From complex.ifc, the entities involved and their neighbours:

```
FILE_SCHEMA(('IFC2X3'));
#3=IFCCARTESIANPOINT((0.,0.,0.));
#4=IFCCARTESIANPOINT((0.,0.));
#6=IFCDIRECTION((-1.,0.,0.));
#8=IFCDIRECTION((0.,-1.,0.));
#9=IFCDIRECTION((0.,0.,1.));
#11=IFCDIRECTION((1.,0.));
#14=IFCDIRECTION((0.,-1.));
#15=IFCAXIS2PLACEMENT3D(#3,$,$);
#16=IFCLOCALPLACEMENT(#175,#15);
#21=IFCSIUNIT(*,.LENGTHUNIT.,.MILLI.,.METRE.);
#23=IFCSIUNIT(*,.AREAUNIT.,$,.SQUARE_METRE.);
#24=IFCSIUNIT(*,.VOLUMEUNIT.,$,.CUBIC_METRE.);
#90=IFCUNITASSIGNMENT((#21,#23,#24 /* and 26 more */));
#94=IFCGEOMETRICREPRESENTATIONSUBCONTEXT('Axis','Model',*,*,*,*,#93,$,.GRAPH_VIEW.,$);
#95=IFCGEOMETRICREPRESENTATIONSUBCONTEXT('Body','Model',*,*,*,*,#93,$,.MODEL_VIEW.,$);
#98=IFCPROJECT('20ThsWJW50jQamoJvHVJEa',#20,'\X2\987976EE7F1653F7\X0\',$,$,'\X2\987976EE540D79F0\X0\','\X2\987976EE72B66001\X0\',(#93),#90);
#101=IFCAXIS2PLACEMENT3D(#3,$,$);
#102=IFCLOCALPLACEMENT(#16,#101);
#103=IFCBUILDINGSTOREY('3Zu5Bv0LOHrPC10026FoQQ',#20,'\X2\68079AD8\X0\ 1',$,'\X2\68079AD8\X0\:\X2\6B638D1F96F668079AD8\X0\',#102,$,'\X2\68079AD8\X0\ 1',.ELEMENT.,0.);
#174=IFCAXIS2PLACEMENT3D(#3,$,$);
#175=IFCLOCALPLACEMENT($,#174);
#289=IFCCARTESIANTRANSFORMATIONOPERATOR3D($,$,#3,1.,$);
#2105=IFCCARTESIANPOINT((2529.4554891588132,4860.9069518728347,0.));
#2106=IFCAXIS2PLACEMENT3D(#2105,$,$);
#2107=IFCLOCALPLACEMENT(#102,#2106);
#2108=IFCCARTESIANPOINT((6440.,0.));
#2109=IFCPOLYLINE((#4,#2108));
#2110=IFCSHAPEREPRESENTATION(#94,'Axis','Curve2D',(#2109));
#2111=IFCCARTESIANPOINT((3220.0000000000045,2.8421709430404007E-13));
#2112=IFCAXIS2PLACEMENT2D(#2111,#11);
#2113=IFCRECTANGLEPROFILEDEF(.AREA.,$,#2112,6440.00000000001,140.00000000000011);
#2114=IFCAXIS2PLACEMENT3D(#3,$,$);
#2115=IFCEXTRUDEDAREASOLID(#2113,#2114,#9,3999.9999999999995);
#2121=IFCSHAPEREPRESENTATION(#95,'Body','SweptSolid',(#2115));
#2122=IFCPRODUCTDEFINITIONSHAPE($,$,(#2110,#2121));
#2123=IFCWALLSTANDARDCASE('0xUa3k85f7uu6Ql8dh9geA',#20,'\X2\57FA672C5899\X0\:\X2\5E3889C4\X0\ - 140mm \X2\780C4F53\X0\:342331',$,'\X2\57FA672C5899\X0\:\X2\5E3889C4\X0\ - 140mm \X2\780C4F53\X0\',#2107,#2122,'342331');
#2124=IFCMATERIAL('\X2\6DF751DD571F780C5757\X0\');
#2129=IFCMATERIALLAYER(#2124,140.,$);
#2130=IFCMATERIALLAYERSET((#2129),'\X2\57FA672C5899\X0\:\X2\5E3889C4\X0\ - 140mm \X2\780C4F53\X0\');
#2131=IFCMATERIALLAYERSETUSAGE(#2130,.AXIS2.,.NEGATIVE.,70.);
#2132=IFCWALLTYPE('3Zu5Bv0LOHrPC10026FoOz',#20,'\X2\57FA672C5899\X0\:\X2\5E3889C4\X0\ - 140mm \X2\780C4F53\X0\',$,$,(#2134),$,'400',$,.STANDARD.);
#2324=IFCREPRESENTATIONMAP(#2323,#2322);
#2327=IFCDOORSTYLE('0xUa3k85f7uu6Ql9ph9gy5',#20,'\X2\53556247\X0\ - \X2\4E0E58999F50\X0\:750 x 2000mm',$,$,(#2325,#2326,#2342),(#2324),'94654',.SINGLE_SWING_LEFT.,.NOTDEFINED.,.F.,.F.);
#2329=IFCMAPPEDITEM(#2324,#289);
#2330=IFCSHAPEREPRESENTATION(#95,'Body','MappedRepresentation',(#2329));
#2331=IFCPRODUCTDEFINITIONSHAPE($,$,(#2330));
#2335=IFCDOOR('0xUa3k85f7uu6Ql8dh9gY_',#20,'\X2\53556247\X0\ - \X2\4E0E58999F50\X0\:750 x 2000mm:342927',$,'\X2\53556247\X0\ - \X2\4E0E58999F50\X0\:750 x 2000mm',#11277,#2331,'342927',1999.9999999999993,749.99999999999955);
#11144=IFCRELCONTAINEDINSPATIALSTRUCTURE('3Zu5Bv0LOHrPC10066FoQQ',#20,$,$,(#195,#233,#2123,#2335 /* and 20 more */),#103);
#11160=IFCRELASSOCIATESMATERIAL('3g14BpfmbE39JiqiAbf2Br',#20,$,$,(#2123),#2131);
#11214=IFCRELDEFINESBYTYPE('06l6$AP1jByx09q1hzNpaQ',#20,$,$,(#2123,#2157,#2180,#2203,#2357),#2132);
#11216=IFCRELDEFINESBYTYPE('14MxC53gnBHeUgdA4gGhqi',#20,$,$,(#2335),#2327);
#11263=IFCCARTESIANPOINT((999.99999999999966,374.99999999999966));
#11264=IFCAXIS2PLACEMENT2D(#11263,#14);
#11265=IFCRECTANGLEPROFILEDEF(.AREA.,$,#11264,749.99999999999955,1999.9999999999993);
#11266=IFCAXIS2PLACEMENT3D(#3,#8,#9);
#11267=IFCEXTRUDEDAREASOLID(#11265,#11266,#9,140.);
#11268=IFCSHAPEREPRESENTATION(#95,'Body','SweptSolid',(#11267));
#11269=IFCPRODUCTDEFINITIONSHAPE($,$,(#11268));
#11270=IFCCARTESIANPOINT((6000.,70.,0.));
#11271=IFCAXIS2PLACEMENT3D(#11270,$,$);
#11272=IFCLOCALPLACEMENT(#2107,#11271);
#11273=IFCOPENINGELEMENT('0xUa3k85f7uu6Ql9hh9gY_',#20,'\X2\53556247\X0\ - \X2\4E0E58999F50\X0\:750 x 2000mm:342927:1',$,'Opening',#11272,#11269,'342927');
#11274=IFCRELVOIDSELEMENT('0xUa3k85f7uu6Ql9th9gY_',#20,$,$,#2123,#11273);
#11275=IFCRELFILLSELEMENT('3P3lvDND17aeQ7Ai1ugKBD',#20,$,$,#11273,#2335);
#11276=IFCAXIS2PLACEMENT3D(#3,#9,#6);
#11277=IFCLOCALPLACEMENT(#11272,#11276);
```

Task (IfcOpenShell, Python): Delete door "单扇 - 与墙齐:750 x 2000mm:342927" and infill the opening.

```python
import ifcopenshell
import ifcopenshell.api.feature
import ifcopenshell.api.root
import ifcopenshell.geom
import ifcopenshell.util.shape

model = ifcopenshell.open("complex.ifc")
settings = ifcopenshell.geom.settings()


def volume(element):
    """Net volume in cubic metres, openings subtracted."""
    shape = ifcopenshell.geom.create_shape(settings, element)
    return ifcopenshell.util.shape.get_volume(shape.geometry)


door = model.by_id(2335)
opening = door.FillsVoids[0].RelatingOpeningElement
wall = opening.VoidsElements[0].RelatingBuildingElement
before = volume(wall)

ifcopenshell.api.root.remove_product(model, product=door)
ifcopenshell.api.feature.remove_feature(model, feature=opening)

after = volume(wall)

print(f"wall volume {before:.3f} -> {after:.3f} m3")

model.write("complex_v2.ifc")
```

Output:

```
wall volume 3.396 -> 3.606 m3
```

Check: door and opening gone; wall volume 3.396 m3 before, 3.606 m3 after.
